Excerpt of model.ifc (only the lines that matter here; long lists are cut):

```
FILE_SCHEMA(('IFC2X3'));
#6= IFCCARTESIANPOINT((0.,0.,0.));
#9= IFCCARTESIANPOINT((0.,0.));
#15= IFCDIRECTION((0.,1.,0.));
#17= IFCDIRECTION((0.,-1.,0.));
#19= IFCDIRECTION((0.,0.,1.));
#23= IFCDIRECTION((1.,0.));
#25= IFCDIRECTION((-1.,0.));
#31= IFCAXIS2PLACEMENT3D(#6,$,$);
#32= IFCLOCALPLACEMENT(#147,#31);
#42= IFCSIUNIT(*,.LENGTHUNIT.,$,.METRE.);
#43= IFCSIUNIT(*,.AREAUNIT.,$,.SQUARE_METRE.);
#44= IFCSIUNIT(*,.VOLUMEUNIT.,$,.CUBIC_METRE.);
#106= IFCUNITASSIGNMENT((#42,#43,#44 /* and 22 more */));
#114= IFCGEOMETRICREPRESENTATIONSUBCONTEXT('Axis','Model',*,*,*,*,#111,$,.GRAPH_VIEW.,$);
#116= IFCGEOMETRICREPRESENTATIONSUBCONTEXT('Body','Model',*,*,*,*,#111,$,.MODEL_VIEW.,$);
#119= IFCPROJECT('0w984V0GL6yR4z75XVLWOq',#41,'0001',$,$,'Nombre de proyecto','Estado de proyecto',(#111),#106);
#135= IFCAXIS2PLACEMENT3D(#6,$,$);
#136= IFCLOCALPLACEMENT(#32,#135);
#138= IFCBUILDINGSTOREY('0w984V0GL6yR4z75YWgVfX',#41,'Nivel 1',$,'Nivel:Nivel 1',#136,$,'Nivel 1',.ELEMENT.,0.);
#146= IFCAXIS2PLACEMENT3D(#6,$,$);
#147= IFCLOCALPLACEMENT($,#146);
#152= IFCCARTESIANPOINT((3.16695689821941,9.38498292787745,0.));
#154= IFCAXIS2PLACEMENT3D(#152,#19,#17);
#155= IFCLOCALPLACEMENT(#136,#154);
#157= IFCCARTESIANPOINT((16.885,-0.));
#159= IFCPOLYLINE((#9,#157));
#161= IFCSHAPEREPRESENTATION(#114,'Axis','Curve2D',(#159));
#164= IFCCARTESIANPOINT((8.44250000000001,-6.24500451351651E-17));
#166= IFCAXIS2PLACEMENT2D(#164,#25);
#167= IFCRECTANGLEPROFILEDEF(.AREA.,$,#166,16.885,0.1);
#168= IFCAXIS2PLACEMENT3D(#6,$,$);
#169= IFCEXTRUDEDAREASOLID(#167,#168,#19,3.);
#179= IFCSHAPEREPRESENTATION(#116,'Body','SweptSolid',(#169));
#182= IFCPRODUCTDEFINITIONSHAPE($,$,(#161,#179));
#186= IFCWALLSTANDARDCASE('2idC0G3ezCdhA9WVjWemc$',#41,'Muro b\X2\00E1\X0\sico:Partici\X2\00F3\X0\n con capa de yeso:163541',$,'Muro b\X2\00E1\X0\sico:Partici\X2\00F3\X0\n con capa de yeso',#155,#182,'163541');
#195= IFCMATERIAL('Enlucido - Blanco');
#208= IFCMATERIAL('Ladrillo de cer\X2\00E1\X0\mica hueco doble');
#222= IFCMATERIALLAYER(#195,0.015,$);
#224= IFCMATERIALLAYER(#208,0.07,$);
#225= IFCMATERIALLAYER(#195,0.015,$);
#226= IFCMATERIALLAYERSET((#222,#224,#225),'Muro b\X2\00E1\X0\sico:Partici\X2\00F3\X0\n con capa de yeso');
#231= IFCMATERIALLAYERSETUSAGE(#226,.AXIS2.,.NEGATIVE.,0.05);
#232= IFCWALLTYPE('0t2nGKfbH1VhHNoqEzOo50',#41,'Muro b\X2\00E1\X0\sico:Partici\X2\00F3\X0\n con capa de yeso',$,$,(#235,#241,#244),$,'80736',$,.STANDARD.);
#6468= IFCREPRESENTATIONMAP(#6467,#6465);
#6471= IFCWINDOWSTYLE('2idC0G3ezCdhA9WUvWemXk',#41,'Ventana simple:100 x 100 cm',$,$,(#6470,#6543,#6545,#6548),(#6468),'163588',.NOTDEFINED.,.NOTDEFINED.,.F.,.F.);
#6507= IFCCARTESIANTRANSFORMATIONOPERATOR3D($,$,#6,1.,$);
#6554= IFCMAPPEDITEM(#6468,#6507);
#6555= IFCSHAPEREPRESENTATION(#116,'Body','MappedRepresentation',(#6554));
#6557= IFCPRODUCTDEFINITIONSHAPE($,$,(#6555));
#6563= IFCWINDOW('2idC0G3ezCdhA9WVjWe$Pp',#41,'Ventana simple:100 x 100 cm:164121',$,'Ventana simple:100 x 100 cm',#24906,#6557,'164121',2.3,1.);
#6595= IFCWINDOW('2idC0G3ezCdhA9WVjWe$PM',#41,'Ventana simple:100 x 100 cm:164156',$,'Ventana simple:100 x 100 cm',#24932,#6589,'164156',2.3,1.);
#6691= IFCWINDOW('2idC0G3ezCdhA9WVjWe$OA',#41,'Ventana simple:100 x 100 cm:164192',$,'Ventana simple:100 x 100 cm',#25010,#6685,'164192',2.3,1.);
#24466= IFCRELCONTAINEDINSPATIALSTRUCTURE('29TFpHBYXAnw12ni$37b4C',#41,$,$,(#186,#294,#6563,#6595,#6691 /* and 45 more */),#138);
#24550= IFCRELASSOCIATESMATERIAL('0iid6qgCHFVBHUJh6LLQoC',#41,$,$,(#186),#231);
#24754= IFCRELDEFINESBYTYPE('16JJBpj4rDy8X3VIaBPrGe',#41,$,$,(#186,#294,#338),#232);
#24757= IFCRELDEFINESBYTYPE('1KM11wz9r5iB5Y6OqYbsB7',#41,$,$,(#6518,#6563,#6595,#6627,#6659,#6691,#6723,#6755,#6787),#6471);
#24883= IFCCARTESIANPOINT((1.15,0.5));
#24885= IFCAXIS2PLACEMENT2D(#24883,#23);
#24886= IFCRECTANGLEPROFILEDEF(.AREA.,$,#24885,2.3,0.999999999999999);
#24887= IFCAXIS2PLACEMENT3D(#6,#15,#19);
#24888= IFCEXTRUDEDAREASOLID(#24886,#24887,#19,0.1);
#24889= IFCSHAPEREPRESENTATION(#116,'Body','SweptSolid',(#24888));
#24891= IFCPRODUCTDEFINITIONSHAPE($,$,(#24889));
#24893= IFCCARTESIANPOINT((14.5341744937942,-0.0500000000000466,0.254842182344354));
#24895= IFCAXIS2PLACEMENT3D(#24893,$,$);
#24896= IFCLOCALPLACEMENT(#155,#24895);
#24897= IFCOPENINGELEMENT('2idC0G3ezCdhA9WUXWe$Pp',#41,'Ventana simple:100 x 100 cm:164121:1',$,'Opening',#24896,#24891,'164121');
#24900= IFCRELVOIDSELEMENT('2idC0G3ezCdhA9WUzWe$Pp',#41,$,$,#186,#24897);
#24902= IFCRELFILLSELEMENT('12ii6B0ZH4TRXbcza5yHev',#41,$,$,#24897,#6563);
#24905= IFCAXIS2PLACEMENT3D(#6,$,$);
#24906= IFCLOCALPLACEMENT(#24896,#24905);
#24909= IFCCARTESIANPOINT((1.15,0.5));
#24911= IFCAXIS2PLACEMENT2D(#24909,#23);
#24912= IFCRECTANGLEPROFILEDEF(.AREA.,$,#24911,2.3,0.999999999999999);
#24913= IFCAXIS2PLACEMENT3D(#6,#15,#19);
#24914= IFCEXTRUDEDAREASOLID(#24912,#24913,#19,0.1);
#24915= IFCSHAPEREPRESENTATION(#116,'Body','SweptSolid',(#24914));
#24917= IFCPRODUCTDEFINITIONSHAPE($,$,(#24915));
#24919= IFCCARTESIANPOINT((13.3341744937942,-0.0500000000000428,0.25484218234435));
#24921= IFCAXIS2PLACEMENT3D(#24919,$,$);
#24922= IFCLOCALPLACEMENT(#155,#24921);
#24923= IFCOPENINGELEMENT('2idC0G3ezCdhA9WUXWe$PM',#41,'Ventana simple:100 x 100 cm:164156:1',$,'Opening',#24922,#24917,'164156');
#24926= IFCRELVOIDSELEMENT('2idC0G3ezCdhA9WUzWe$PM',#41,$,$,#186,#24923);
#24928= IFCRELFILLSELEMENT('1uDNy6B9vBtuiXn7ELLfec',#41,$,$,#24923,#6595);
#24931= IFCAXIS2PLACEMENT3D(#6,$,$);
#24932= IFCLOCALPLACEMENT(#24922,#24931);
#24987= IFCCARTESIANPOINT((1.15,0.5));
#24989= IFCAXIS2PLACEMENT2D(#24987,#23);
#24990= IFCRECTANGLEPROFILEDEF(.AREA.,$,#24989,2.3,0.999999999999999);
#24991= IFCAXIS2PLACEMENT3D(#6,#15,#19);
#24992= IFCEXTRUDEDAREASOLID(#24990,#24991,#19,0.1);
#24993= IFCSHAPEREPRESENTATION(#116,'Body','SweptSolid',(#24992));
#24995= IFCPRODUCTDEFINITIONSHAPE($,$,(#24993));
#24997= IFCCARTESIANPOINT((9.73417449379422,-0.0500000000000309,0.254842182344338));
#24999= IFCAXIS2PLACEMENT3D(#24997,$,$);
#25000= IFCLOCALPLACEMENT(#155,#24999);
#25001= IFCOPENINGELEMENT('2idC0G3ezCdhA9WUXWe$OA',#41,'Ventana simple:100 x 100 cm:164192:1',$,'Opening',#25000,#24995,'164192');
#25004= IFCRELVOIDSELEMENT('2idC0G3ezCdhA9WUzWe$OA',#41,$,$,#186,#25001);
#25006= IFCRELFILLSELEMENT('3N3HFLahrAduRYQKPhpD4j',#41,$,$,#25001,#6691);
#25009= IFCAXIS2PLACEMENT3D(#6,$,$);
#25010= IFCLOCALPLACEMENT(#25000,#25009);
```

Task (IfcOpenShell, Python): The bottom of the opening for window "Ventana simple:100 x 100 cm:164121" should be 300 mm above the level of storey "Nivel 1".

```python
import numpy as np
import ifcopenshell
import ifcopenshell.api.geometry
import ifcopenshell.geom
import ifcopenshell.util.element
import ifcopenshell.util.placement
import ifcopenshell.util.shape
import ifcopenshell.util.unit

model = ifcopenshell.open("model.ifc")
unit_scale = ifcopenshell.util.unit.calculate_unit_scale(model)

window = model.by_guid("2idC0G3ezCdhA9WVjWe$Pp")
opening = window.FillsVoids[0].RelatingOpeningElement
storey = ifcopenshell.util.element.get_container(window, ifc_class="IfcBuildingStorey")
level = ifcopenshell.util.placement.get_local_placement(storey.ObjectPlacement)[2, 3]

# The opening's origin need not be at the sill, so measure its lowest point.
shape = ifcopenshell.geom.create_shape(ifcopenshell.geom.settings(), opening)
bottom = ifcopenshell.util.shape.get_shape_bottom_elevation(shape, shape.geometry) / unit_scale
dz = level + 0.3 / unit_scale - bottom

shift = np.array([0.0, 0.0, dz])
# The window is placed relative to its opening, so it follows when the opening moves.
matrix = ifcopenshell.util.placement.get_local_placement(opening.ObjectPlacement)
matrix[:3, 3] += shift
ifcopenshell.api.geometry.edit_object_placement(
    model, product=opening, matrix=matrix, is_si=False, should_transform_children=True
)

print(f"moved by {dz * unit_scale:+.3f} m")

model.write("model_rev.ifc")
```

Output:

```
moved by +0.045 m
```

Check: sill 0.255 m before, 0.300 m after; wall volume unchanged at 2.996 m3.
